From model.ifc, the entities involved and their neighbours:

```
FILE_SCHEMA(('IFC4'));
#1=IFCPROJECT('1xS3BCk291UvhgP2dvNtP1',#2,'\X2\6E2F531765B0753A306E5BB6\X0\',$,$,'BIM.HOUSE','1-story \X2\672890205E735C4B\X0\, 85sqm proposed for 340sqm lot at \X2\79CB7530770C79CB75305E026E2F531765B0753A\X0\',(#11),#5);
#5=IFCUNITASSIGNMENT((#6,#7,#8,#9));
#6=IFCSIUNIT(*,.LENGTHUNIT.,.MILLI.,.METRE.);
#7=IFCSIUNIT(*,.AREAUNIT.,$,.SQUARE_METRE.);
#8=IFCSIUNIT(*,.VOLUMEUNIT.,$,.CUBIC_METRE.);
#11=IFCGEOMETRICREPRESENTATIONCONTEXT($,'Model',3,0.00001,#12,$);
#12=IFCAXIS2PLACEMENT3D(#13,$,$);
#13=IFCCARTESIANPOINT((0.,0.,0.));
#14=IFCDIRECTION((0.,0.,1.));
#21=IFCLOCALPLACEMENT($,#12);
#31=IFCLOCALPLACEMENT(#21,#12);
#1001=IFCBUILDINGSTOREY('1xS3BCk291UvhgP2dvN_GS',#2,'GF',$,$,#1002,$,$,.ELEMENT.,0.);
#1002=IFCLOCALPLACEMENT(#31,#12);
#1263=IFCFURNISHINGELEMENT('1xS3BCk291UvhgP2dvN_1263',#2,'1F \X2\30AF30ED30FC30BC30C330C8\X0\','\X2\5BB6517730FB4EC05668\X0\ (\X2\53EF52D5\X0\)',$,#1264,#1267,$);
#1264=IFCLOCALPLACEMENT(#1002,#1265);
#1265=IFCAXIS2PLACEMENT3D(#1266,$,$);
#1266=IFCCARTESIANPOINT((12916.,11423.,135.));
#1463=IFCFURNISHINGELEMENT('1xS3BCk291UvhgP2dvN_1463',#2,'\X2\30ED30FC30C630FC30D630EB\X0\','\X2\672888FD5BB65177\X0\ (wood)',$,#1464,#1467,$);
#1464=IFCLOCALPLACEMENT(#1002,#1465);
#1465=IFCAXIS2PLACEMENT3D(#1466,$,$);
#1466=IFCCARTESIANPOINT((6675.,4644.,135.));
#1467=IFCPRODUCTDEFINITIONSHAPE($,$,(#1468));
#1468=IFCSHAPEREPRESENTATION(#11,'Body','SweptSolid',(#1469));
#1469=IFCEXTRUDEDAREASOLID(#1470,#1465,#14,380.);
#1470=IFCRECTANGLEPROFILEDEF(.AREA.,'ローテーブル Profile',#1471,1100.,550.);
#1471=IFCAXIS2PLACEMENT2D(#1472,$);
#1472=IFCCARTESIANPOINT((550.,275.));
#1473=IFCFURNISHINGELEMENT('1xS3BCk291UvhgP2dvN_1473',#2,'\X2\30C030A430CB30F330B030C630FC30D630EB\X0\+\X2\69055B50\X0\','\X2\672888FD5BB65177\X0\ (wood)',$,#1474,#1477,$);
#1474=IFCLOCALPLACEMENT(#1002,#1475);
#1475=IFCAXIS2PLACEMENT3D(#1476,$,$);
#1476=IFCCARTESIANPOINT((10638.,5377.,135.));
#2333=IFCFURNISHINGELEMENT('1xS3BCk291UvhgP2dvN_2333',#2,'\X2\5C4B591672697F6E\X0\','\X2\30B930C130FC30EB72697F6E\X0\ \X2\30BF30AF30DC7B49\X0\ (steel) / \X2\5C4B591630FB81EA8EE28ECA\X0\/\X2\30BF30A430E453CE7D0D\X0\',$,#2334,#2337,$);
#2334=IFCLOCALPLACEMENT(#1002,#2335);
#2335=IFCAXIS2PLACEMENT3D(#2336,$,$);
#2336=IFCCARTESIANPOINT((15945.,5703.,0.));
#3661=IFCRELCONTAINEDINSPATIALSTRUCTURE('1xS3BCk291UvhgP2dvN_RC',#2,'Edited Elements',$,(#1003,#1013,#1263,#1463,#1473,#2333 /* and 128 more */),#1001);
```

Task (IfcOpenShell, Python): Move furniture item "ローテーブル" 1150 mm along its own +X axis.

```python
import ifcopenshell
import ifcopenshell.api.geometry
import ifcopenshell.util.placement
import ifcopenshell.util.unit

model = ifcopenshell.open("model.ifc")
unit_scale = ifcopenshell.util.unit.calculate_unit_scale(model)

item = model.by_guid("1xS3BCk291UvhgP2dvN_1463")
matrix = ifcopenshell.util.placement.get_local_placement(item.ObjectPlacement)
matrix[:3, 3] += matrix[:3, 0] * 1.15 / unit_scale
ifcopenshell.api.geometry.edit_object_placement(model, product=item, matrix=matrix, is_si=False)

print(ifcopenshell.util.placement.get_local_placement(item.ObjectPlacement).round(3) + 0.0)

model.write("model_edited.ifc")
```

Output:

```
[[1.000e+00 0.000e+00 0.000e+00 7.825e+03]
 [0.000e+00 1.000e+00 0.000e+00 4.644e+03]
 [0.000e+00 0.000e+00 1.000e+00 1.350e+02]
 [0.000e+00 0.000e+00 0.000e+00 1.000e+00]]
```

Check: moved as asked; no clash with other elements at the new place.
